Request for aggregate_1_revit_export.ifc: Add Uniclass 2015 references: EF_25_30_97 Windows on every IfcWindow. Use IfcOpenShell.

First a look at what the model holds.

```python
import ifcopenshell

model = ifcopenshell.open("aggregate_1_revit_export.ifc")
print(model.schema)
print("classifications:", [c.Name for c in model.by_type("IfcClassification")])
for ifc_class in ("IfcDoor", "IfcRoof", "IfcStair", "IfcWall", "IfcWindow"):
    print(ifc_class, len(model.by_type(ifc_class)))
```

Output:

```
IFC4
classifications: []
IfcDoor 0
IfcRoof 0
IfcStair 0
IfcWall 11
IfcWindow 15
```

```python
import ifcopenshell
import ifcopenshell.api.classification

model = ifcopenshell.open("aggregate_1_revit_export.ifc")

system = ifcopenshell.api.classification.add_classification(model, classification="Uniclass 2015")

codes = {
    "IfcWindow": ("EF_25_30_97", "Windows"),
}
for ifc_class, (code, name) in codes.items():
    products = model.by_type(ifc_class)
    ifcopenshell.api.classification.add_reference(
        model, products=products, classification=system, identification=code, name=name
    )
    print(code, len(products))

model.write("aggregate_1_revit_export_updated.ifc")
```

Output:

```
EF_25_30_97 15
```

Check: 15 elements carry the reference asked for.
